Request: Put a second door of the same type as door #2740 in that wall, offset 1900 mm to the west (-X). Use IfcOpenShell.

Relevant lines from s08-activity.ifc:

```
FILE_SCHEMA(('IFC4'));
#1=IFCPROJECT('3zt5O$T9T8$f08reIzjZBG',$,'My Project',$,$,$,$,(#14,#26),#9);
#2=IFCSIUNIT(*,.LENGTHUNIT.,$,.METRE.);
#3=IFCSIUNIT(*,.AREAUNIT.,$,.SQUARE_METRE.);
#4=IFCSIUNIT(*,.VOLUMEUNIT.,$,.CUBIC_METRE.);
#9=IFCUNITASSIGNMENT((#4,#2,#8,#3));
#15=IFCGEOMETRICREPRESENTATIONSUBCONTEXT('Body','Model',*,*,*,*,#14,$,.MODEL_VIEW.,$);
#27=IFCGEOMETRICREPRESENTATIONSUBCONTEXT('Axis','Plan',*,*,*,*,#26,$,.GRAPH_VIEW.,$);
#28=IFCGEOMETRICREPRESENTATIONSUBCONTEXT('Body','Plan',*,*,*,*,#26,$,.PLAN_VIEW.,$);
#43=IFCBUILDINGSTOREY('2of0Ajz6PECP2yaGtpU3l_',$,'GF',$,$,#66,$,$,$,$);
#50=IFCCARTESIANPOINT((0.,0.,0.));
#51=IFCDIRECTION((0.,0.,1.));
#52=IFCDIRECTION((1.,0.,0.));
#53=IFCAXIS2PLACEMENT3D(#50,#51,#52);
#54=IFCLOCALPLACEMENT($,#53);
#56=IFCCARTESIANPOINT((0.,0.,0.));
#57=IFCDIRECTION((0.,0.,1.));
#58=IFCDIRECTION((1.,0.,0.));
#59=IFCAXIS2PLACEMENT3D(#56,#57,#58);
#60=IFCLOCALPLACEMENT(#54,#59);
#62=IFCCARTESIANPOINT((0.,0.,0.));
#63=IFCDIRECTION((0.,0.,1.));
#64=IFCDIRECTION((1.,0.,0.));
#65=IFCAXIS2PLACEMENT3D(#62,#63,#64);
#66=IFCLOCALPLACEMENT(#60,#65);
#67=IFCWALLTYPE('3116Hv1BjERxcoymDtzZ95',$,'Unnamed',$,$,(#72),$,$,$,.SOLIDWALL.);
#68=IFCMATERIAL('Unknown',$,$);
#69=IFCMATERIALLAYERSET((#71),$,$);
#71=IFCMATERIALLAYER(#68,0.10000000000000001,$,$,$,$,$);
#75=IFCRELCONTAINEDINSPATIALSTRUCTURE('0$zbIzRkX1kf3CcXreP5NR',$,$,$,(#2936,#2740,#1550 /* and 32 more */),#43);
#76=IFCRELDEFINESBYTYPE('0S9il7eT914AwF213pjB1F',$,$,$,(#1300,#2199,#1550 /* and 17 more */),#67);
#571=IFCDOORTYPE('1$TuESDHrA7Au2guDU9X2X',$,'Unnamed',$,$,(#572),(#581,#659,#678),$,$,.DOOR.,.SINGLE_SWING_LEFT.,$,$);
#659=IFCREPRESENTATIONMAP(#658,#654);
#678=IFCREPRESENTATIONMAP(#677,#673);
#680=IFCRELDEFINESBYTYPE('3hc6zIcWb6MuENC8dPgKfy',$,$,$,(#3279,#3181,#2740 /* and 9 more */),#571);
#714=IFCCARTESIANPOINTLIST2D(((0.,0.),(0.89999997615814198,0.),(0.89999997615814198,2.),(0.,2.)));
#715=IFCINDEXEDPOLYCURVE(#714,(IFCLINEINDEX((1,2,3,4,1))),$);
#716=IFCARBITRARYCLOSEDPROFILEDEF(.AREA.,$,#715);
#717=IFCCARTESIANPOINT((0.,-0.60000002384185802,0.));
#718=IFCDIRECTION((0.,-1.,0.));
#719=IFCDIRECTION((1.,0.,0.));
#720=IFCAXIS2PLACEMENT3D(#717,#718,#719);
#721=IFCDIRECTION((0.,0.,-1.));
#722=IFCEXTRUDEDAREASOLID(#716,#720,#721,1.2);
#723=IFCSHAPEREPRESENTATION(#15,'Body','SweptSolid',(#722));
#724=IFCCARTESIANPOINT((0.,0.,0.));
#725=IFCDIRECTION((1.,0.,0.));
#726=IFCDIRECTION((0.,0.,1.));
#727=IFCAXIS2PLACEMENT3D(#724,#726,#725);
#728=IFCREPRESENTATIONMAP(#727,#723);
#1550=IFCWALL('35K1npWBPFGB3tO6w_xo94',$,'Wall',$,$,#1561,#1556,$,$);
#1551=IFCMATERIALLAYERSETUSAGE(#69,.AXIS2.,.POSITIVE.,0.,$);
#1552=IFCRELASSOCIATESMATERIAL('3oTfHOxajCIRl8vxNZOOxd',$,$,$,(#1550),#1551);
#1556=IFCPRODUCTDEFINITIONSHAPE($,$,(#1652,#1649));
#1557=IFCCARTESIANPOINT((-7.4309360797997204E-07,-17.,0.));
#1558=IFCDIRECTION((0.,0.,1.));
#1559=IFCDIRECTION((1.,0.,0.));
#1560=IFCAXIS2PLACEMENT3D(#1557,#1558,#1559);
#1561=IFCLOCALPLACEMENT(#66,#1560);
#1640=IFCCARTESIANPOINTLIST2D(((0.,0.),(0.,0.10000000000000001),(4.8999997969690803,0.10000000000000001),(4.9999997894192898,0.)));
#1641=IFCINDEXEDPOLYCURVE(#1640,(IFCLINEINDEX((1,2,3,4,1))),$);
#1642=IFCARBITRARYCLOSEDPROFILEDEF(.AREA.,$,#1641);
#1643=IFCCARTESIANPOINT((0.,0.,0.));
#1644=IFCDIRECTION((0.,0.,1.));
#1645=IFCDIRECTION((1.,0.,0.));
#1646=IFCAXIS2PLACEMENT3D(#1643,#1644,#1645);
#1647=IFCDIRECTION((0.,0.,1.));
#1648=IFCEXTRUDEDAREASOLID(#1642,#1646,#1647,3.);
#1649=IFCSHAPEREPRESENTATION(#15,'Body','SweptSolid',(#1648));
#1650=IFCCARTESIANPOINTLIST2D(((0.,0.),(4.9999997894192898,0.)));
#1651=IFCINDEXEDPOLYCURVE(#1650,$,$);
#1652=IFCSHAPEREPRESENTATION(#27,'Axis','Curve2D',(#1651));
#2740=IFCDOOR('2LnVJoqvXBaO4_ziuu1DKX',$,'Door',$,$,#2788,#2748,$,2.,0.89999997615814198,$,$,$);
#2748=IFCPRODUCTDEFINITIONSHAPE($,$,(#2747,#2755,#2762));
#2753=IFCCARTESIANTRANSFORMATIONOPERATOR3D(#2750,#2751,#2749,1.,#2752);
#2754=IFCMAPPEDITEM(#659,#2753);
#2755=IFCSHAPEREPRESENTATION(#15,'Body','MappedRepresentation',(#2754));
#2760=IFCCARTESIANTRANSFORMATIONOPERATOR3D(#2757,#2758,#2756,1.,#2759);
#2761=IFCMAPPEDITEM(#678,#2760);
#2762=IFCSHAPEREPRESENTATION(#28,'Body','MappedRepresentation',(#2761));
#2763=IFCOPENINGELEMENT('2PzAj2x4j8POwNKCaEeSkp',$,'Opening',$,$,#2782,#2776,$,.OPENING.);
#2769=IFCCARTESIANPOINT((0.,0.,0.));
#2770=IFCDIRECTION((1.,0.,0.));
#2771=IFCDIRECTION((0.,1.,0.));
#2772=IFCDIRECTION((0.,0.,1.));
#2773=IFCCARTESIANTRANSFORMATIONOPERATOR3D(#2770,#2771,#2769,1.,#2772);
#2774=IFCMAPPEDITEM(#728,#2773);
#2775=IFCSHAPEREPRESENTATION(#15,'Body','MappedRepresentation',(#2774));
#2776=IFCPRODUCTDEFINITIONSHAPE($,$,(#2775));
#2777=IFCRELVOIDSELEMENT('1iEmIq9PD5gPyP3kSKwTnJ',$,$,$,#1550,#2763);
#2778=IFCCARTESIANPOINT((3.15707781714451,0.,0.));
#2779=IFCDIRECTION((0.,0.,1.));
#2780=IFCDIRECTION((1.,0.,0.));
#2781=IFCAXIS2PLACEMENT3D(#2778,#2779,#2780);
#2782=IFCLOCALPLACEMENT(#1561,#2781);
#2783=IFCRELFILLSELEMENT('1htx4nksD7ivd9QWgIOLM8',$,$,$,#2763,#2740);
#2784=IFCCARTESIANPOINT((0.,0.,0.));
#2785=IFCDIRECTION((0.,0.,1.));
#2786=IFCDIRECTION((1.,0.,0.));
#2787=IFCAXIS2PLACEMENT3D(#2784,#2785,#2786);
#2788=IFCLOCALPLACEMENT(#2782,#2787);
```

```python
import ifcopenshell
import ifcopenshell.api.feature
import ifcopenshell.api.geometry
import ifcopenshell.api.root
import ifcopenshell.geom
import ifcopenshell.util.element
import ifcopenshell.util.placement
import ifcopenshell.util.shape
import ifcopenshell.util.unit

model = ifcopenshell.open("s08-activity.ifc")
unit_scale = ifcopenshell.util.unit.calculate_unit_scale(model)
settings = ifcopenshell.geom.settings()


def volume(element):
    """Net volume in cubic metres, openings subtracted."""
    shape = ifcopenshell.geom.create_shape(settings, element)
    return ifcopenshell.util.shape.get_volume(shape.geometry)


door = model.by_id(2740)
opening = door.FillsVoids[0].RelatingOpeningElement
wall = opening.VoidsElements[0].RelatingBuildingElement
before = volume(wall)
shift = ifcopenshell.util.placement.get_local_placement(wall.ObjectPlacement)[:3, 0] * -1.9 / unit_scale

# copy_class copies the void relationship, type, container and properties, but no geometry.
new_opening = ifcopenshell.api.root.copy_class(model, product=opening)
new_opening.Representation = ifcopenshell.util.element.copy_deep(
    model, opening.Representation, exclude=["IfcGeometricRepresentationContext", "IfcRepresentationMap"]
)
new_door = ifcopenshell.api.root.copy_class(model, product=door)
new_door.Representation = ifcopenshell.util.element.copy_deep(
    model, door.Representation, exclude=["IfcGeometricRepresentationContext", "IfcRepresentationMap"]
)
ifcopenshell.api.feature.add_filling(model, opening=new_opening, element=new_door)

for old, new in ((opening, new_opening), (door, new_door)):
    matrix = ifcopenshell.util.placement.get_local_placement(old.ObjectPlacement)
    matrix[:3, 3] += shift
    ifcopenshell.api.geometry.edit_object_placement(model, product=new, matrix=matrix, is_si=False)

after = volume(wall)

print(f"wall volume {before:.3f} -> {after:.3f} m3")

model.write("s08-activity-out.ifc")
```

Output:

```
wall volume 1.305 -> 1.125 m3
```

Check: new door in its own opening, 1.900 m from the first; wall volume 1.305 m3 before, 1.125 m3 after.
